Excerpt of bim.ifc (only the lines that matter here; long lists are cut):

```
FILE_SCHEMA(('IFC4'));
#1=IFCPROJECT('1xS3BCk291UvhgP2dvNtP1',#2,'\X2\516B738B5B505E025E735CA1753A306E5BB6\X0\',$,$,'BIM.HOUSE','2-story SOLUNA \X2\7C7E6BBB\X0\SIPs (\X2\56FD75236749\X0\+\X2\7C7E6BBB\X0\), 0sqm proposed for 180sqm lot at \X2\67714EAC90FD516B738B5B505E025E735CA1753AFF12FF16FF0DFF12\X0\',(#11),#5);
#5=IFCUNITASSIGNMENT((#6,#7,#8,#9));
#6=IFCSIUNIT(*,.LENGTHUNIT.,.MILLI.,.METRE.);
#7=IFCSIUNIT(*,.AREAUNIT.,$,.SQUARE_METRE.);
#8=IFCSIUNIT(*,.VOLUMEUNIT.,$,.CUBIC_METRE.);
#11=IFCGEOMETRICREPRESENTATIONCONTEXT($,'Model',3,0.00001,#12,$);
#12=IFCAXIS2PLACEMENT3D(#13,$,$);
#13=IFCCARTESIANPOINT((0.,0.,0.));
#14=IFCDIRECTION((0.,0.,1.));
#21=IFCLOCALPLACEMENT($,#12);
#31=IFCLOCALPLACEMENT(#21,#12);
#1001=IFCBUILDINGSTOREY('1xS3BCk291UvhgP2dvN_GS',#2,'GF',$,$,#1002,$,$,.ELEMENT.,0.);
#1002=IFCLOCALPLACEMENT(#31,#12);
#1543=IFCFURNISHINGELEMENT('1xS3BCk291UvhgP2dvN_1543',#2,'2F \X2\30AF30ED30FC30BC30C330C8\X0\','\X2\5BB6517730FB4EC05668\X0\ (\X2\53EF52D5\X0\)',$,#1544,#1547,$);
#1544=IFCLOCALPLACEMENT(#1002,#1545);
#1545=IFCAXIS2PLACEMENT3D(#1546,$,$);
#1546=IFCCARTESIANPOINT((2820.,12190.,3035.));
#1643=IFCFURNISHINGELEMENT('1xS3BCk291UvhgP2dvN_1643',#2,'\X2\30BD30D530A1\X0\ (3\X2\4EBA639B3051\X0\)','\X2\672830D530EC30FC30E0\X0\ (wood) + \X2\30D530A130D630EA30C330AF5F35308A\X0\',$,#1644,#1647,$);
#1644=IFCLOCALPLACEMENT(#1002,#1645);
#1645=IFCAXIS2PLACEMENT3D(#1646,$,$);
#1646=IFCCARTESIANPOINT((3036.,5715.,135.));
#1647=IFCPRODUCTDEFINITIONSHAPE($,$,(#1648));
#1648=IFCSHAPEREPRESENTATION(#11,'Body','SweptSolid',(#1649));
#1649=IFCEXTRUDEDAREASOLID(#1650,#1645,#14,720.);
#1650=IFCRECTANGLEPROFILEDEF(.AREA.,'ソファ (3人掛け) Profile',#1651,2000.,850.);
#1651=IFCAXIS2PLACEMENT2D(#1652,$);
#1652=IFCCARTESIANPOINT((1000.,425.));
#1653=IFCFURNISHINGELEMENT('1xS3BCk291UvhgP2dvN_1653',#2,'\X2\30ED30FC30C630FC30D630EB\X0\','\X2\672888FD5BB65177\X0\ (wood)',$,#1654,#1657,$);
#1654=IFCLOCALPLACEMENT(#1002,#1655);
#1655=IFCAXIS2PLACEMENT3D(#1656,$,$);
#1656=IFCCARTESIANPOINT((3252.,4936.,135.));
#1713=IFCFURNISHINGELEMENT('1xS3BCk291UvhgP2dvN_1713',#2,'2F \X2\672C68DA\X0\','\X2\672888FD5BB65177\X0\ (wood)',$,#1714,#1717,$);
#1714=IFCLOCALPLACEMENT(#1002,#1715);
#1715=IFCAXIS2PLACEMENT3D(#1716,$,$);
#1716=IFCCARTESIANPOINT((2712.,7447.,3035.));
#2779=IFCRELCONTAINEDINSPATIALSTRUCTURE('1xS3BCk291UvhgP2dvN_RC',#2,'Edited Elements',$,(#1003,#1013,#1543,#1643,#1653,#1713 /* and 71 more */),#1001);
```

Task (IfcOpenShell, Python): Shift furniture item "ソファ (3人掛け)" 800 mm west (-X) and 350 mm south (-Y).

```python
import ifcopenshell
import ifcopenshell.api.geometry
import ifcopenshell.util.placement
import ifcopenshell.util.unit

model = ifcopenshell.open("bim.ifc")
unit_scale = ifcopenshell.util.unit.calculate_unit_scale(model)

item = model.by_id(1643)
matrix = ifcopenshell.util.placement.get_local_placement(item.ObjectPlacement)
matrix[0, 3] -= 0.8 / unit_scale
matrix[1, 3] -= 0.35 / unit_scale
ifcopenshell.api.geometry.edit_object_placement(model, product=item, matrix=matrix, is_si=False)

print(ifcopenshell.util.placement.get_local_placement(item.ObjectPlacement).round(3) + 0.0)

model.write("bim_edited.ifc")
```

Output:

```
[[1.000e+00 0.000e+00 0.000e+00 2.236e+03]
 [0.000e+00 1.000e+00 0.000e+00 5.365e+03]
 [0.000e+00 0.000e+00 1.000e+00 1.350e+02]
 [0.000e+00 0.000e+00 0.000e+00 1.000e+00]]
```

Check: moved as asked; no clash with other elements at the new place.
